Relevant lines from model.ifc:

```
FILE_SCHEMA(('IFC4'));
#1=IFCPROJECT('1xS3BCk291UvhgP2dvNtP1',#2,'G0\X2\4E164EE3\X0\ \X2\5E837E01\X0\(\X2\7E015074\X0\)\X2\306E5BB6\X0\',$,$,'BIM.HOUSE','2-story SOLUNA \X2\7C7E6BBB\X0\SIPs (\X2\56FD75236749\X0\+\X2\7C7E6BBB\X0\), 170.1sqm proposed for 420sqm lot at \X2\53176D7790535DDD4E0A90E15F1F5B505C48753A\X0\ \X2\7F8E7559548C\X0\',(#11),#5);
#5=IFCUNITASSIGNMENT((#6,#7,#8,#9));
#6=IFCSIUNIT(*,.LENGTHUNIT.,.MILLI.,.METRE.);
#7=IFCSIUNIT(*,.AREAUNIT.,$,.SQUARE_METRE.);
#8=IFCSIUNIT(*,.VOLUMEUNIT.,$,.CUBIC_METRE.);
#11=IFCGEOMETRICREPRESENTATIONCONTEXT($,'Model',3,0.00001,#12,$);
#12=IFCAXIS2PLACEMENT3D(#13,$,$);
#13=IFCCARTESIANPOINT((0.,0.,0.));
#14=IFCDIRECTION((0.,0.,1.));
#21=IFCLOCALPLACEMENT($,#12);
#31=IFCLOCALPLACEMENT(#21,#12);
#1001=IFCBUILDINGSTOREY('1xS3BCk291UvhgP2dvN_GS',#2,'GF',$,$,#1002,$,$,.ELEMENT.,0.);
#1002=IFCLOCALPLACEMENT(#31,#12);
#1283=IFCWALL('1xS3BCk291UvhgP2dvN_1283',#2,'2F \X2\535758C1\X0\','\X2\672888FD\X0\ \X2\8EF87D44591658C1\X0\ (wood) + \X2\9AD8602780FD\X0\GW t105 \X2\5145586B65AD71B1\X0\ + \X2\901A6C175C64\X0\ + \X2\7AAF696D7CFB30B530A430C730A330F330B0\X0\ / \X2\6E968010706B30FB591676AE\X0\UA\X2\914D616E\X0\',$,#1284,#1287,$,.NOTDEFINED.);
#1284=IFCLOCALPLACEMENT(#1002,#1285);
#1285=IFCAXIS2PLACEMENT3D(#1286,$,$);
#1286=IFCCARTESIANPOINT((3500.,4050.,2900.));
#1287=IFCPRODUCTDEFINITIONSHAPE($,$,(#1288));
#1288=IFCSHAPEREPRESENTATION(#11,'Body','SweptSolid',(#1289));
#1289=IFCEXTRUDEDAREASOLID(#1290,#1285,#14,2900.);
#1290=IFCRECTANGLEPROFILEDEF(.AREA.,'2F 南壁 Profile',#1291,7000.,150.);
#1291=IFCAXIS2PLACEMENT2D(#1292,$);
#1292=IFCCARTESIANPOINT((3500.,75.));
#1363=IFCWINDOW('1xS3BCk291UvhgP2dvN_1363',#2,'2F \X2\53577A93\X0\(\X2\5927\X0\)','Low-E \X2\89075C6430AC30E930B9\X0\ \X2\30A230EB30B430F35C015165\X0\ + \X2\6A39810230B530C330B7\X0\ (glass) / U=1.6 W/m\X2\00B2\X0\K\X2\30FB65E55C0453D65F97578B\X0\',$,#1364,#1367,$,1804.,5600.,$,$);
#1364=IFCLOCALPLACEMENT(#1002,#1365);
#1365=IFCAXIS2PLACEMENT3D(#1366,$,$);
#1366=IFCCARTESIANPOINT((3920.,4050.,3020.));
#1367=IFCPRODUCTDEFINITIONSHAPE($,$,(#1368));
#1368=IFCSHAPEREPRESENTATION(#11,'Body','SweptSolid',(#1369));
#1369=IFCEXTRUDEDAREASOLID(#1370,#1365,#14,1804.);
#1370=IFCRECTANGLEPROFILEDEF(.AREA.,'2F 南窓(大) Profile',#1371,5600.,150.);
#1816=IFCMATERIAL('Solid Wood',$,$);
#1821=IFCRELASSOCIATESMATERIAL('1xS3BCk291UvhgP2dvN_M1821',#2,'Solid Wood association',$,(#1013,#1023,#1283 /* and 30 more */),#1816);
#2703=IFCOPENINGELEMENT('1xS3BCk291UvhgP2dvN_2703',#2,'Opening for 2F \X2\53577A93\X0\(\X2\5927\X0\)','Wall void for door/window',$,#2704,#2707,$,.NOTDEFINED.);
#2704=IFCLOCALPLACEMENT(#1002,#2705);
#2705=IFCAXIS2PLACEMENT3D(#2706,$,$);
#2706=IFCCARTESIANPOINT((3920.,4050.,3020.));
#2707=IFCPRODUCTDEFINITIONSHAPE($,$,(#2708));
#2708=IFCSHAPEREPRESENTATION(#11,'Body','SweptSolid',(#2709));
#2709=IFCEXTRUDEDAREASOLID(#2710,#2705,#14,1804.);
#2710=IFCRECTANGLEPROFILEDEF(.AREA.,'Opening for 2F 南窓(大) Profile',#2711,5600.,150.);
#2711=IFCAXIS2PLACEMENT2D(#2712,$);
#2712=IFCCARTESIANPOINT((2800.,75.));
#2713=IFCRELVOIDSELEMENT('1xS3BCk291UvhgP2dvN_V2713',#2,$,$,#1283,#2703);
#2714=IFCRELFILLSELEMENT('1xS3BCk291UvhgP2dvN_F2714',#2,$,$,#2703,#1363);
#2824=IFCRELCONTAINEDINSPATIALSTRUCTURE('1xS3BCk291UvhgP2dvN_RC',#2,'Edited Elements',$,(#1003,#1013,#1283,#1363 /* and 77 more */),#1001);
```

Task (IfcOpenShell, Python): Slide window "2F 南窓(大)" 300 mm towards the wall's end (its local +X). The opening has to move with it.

```python
import ifcopenshell
import ifcopenshell.api.geometry
import ifcopenshell.util.placement

model = ifcopenshell.open("model.ifc")

window = model.by_guid("1xS3BCk291UvhgP2dvN_1363")
opening = window.FillsVoids[0].RelatingOpeningElement
wall = opening.VoidsElements[0].RelatingBuildingElement

wall_matrix = ifcopenshell.util.placement.get_local_placement(wall.ObjectPlacement)
shift = wall_matrix[:3, 0] * 300.0
before = ifcopenshell.util.placement.get_local_placement(window.ObjectPlacement)[:3, 3].copy()

# The window is not placed relative to its opening, so move both.
for product in (opening, window):
    matrix = ifcopenshell.util.placement.get_local_placement(product.ObjectPlacement)
    matrix[:3, 3] += shift
    ifcopenshell.api.geometry.edit_object_placement(model, product=product, matrix=matrix, is_si=False)

after = ifcopenshell.util.placement.get_local_placement(window.ObjectPlacement)[:3, 3]
print("window moved by", (after - before).round(3) + 0.0)

model.write("model_v2.ifc")
```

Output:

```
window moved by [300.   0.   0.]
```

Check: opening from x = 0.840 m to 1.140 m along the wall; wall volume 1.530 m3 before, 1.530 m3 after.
